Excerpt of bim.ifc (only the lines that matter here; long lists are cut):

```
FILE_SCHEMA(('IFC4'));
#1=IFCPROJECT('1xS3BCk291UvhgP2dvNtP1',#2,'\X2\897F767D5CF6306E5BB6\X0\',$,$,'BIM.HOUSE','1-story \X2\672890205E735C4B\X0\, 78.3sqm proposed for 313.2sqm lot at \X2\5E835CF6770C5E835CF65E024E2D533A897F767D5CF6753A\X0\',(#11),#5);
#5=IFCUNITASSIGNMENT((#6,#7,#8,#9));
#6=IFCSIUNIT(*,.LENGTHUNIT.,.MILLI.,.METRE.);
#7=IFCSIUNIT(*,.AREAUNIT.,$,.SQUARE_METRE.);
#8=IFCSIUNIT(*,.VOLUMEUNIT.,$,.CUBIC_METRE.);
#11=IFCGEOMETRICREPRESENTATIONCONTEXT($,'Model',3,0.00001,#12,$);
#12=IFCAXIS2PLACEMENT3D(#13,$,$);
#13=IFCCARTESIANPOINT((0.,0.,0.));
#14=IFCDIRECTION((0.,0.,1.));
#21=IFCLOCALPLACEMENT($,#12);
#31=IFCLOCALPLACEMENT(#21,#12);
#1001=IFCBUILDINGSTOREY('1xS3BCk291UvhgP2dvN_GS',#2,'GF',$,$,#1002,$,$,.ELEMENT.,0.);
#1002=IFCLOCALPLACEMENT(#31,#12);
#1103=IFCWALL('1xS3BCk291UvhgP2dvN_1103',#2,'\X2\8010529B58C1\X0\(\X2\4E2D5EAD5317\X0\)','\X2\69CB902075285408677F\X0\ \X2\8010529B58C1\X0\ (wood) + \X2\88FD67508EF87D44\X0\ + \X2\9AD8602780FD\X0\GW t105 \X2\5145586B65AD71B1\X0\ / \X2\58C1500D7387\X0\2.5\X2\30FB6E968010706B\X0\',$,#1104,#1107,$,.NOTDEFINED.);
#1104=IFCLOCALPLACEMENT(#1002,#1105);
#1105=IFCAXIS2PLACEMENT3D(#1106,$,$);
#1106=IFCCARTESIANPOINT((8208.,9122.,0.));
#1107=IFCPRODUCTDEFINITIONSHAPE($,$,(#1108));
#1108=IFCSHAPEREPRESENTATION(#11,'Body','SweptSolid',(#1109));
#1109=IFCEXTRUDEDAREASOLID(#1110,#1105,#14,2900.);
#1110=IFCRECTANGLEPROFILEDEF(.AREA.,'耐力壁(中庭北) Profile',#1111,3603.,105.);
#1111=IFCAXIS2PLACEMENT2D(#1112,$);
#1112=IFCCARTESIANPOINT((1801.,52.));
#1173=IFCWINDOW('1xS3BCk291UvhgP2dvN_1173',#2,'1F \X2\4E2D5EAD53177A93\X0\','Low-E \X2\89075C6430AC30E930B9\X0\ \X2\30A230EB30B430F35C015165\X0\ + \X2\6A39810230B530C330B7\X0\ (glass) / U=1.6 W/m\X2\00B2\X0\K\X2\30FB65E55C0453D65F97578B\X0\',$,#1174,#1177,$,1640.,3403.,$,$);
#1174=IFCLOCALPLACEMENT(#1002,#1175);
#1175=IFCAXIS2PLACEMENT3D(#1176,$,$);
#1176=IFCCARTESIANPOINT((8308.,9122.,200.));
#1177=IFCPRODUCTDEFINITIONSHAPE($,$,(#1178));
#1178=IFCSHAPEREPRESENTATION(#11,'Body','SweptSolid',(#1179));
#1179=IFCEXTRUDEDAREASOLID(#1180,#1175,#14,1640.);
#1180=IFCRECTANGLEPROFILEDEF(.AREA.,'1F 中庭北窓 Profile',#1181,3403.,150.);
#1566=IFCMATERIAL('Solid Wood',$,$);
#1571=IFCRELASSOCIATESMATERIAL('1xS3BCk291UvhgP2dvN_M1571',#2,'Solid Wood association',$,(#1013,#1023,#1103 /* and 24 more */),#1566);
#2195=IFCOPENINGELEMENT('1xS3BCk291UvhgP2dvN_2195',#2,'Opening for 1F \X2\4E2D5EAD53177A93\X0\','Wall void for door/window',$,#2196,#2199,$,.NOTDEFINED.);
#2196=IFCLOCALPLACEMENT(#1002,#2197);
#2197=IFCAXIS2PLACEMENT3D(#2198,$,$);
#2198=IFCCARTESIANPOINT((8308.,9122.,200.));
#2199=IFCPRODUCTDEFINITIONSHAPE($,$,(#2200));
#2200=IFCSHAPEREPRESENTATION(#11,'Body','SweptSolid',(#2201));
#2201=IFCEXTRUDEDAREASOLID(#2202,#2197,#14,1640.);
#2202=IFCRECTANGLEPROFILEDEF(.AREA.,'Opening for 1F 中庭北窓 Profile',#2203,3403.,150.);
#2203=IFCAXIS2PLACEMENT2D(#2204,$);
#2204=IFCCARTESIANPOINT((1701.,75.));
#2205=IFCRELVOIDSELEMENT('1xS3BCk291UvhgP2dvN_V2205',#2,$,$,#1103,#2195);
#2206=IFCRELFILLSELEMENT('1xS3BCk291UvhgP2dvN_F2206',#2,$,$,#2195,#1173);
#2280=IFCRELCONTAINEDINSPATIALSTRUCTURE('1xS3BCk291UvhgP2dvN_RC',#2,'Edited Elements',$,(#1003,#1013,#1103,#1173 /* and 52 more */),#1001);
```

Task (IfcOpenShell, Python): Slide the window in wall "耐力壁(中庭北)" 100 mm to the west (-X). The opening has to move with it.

```python
import ifcopenshell
import ifcopenshell.api.geometry
import ifcopenshell.util.placement
import ifcopenshell.util.unit

model = ifcopenshell.open("bim.ifc")
unit_scale = ifcopenshell.util.unit.calculate_unit_scale(model)

window = model.by_guid("1xS3BCk291UvhgP2dvN_1173")
opening = window.FillsVoids[0].RelatingOpeningElement
wall = opening.VoidsElements[0].RelatingBuildingElement

wall_matrix = ifcopenshell.util.placement.get_local_placement(wall.ObjectPlacement)
shift = wall_matrix[:3, 0] * -0.1 / unit_scale
before = ifcopenshell.util.placement.get_local_placement(window.ObjectPlacement)[:3, 3].copy()

# The window is not placed relative to its opening, so move both.
for product in (opening, window):
    matrix = ifcopenshell.util.placement.get_local_placement(product.ObjectPlacement)
    matrix[:3, 3] += shift
    ifcopenshell.api.geometry.edit_object_placement(model, product=product, matrix=matrix, is_si=False)

after = ifcopenshell.util.placement.get_local_placement(window.ObjectPlacement)[:3, 3]
print("window moved by", (after - before).round(3) + 0.0)

model.write("bim_updated.ifc")
```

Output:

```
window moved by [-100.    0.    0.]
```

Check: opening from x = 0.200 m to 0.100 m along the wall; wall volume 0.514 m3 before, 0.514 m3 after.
